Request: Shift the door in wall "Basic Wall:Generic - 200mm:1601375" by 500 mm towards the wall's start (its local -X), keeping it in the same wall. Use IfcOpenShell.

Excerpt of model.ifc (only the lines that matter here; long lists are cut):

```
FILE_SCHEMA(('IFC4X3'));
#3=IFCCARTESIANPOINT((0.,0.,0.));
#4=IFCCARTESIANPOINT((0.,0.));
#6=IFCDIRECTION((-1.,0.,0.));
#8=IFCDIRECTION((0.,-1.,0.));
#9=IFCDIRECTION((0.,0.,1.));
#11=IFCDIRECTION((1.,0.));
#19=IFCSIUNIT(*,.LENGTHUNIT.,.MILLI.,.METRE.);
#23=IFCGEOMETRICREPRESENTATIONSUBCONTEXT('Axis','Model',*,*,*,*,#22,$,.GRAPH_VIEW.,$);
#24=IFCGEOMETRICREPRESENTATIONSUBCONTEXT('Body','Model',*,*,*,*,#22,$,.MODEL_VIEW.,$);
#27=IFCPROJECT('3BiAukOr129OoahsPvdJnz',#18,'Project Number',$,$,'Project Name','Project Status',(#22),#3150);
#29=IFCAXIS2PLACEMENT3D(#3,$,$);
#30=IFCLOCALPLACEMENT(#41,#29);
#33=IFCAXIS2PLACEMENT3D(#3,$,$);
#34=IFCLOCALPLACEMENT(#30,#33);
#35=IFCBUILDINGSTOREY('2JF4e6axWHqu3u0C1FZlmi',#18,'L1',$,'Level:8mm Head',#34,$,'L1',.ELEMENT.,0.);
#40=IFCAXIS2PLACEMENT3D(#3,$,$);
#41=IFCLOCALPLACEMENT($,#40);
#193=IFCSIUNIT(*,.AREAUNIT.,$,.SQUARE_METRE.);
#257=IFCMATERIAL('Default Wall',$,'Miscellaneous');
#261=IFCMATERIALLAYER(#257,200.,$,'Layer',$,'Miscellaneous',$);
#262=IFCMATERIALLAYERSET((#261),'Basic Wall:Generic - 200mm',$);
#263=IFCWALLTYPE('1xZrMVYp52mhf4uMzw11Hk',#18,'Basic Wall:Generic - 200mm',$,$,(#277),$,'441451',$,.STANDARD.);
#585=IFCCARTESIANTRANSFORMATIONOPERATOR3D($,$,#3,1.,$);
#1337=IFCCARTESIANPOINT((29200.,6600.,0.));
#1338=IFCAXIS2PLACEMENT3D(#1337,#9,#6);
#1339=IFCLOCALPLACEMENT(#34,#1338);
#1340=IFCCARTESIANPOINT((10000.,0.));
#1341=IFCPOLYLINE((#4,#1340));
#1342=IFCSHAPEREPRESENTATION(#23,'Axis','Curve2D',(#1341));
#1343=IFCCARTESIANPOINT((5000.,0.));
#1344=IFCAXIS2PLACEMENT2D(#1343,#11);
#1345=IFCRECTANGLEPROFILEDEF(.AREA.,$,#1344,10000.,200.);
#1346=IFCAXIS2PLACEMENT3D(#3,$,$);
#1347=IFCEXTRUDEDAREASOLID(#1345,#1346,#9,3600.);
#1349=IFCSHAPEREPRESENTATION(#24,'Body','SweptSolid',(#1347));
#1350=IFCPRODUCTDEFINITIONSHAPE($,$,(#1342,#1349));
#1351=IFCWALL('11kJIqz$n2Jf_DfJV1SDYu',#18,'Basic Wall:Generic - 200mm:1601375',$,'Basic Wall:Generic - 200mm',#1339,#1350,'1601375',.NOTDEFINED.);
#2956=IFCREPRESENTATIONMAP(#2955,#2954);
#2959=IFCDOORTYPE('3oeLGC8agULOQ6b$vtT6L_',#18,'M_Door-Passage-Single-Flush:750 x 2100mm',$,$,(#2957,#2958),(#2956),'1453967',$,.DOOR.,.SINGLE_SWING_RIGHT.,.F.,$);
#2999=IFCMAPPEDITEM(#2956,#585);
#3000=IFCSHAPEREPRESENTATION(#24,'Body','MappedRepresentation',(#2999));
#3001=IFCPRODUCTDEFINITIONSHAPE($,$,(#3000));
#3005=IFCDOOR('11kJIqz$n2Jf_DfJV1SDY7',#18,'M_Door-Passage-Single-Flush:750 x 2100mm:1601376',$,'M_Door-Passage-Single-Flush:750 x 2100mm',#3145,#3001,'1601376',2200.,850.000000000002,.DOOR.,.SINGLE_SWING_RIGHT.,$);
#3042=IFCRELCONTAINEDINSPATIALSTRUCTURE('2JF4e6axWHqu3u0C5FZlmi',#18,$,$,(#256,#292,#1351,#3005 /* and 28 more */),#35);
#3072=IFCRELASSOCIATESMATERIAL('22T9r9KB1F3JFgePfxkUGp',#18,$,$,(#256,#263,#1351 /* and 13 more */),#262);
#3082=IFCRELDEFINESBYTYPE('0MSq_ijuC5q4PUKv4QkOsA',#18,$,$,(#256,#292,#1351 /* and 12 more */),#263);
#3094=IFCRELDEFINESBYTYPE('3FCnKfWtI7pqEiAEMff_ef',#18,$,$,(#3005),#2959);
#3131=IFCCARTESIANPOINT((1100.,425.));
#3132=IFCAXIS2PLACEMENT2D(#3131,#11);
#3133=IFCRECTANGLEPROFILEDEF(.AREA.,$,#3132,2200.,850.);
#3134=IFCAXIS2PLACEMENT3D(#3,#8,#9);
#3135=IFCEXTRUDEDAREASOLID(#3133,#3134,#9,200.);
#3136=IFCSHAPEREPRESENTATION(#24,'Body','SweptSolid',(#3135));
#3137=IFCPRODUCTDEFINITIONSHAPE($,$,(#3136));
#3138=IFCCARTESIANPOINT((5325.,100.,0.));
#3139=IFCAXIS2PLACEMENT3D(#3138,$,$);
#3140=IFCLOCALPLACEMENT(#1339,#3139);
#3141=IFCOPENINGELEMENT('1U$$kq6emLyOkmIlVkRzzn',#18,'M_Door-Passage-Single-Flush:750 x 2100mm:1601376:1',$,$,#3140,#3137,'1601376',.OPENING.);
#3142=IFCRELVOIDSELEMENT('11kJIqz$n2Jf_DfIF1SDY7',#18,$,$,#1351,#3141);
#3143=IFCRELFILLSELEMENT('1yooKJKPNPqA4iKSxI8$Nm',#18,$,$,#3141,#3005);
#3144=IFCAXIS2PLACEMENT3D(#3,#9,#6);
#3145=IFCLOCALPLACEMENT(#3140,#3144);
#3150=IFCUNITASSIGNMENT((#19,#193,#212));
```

```python
import ifcopenshell
import ifcopenshell.api.geometry
import ifcopenshell.util.placement

model = ifcopenshell.open("model.ifc")

door = model.by_guid("11kJIqz$n2Jf_DfJV1SDY7")
opening = door.FillsVoids[0].RelatingOpeningElement
wall = opening.VoidsElements[0].RelatingBuildingElement

wall_matrix = ifcopenshell.util.placement.get_local_placement(wall.ObjectPlacement)
shift = wall_matrix[:3, 0] * -500.0
before = ifcopenshell.util.placement.get_local_placement(door.ObjectPlacement)[:3, 3].copy()

# The door is placed relative to its opening, so it follows when the opening moves.
matrix = ifcopenshell.util.placement.get_local_placement(opening.ObjectPlacement)
matrix[:3, 3] += shift
ifcopenshell.api.geometry.edit_object_placement(
    model, product=opening, matrix=matrix, is_si=False, should_transform_children=True
)

after = ifcopenshell.util.placement.get_local_placement(door.ObjectPlacement)[:3, 3]
print("door moved by", (after - before).round(3) + 0.0)

model.write("model_rev.ifc")
```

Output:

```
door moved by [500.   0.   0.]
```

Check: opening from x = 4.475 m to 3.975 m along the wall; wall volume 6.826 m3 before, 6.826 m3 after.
